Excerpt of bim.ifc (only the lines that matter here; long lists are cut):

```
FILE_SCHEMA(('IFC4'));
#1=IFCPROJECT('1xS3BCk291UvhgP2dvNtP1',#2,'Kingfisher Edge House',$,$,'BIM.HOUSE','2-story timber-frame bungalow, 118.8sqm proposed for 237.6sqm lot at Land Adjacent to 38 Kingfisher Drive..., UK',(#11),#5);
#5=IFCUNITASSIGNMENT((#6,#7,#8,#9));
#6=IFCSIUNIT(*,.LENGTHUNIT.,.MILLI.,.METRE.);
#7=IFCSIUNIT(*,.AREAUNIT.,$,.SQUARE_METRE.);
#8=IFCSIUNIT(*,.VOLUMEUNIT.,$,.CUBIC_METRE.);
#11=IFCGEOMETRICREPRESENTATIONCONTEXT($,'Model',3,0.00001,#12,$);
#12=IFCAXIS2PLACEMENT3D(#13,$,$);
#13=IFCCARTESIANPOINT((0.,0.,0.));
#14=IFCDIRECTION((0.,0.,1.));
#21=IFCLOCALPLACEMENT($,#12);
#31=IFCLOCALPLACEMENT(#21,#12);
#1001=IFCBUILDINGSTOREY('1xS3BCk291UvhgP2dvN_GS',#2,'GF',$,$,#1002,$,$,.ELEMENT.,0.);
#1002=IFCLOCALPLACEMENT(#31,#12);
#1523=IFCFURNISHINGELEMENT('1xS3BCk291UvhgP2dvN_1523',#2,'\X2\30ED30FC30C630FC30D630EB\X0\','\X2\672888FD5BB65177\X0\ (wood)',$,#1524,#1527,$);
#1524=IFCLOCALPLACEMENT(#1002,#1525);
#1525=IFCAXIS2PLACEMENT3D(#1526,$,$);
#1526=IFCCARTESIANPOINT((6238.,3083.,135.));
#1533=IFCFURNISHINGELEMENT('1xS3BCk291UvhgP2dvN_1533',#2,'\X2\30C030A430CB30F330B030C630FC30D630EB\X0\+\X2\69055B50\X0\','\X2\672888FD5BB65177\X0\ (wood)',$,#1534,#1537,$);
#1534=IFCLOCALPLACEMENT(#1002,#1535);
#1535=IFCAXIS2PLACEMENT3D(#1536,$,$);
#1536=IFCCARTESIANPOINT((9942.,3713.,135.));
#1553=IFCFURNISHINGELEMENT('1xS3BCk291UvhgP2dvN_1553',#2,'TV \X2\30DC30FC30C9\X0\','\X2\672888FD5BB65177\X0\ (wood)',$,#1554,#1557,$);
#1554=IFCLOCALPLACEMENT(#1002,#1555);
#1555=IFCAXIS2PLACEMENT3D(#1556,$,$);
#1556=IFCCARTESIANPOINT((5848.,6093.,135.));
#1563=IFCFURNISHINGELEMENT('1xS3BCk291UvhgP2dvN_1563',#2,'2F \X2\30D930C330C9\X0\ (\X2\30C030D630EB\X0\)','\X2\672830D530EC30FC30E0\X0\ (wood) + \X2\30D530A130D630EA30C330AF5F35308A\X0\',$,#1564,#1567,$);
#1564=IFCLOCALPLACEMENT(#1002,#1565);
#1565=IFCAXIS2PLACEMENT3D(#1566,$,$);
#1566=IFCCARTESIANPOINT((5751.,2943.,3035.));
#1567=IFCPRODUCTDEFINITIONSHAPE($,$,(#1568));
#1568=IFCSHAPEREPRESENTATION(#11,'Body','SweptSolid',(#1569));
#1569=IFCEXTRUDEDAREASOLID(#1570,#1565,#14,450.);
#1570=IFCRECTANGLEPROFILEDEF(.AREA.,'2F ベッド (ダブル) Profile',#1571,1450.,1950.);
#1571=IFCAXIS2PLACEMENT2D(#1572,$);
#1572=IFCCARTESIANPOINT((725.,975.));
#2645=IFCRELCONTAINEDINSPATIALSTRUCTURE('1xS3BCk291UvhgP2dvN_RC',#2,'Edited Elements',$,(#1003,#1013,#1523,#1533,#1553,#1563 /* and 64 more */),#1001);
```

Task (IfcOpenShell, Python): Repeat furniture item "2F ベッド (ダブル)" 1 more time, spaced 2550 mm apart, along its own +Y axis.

```python
import ifcopenshell
import ifcopenshell.api.geometry
import ifcopenshell.api.root
import ifcopenshell.util.element
import ifcopenshell.util.placement
import ifcopenshell.util.unit

model = ifcopenshell.open("bim.ifc")
unit_scale = ifcopenshell.util.unit.calculate_unit_scale(model)


def reuse_history(source, copy):
    """copy_class also copies each property set's owner history, people and application; keep the originals."""
    for rel in copy.IsDefinedBy:
        if rel.is_a("IfcRelDefinesByProperties") and (history := rel.RelatingPropertyDefinition.OwnerHistory):
            rel.RelatingPropertyDefinition.OwnerHistory = source.OwnerHistory
            ifcopenshell.util.element.remove_deep2(model, history)


source = model.by_guid("1xS3BCk291UvhgP2dvN_1563")
base = ifcopenshell.util.placement.get_local_placement(source.ObjectPlacement)
step = base[:3, 1] * 2.55 / unit_scale

for i in range(1, 2):
    copy = ifcopenshell.api.root.copy_class(model, product=source)
    copy.Representation = ifcopenshell.util.element.copy_deep(
        model, source.Representation, exclude=["IfcGeometricRepresentationContext", "IfcRepresentationMap"]
    )
    reuse_history(source, copy)
    matrix = base.copy()
    matrix[:3, 3] += i * step
    print("added at", matrix[:3, 3].round(3) + 0.0)
    ifcopenshell.api.geometry.edit_object_placement(model, product=copy, matrix=matrix, is_si=False)

model.write("bim_updated.ifc")
```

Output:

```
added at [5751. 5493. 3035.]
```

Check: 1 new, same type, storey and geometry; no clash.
